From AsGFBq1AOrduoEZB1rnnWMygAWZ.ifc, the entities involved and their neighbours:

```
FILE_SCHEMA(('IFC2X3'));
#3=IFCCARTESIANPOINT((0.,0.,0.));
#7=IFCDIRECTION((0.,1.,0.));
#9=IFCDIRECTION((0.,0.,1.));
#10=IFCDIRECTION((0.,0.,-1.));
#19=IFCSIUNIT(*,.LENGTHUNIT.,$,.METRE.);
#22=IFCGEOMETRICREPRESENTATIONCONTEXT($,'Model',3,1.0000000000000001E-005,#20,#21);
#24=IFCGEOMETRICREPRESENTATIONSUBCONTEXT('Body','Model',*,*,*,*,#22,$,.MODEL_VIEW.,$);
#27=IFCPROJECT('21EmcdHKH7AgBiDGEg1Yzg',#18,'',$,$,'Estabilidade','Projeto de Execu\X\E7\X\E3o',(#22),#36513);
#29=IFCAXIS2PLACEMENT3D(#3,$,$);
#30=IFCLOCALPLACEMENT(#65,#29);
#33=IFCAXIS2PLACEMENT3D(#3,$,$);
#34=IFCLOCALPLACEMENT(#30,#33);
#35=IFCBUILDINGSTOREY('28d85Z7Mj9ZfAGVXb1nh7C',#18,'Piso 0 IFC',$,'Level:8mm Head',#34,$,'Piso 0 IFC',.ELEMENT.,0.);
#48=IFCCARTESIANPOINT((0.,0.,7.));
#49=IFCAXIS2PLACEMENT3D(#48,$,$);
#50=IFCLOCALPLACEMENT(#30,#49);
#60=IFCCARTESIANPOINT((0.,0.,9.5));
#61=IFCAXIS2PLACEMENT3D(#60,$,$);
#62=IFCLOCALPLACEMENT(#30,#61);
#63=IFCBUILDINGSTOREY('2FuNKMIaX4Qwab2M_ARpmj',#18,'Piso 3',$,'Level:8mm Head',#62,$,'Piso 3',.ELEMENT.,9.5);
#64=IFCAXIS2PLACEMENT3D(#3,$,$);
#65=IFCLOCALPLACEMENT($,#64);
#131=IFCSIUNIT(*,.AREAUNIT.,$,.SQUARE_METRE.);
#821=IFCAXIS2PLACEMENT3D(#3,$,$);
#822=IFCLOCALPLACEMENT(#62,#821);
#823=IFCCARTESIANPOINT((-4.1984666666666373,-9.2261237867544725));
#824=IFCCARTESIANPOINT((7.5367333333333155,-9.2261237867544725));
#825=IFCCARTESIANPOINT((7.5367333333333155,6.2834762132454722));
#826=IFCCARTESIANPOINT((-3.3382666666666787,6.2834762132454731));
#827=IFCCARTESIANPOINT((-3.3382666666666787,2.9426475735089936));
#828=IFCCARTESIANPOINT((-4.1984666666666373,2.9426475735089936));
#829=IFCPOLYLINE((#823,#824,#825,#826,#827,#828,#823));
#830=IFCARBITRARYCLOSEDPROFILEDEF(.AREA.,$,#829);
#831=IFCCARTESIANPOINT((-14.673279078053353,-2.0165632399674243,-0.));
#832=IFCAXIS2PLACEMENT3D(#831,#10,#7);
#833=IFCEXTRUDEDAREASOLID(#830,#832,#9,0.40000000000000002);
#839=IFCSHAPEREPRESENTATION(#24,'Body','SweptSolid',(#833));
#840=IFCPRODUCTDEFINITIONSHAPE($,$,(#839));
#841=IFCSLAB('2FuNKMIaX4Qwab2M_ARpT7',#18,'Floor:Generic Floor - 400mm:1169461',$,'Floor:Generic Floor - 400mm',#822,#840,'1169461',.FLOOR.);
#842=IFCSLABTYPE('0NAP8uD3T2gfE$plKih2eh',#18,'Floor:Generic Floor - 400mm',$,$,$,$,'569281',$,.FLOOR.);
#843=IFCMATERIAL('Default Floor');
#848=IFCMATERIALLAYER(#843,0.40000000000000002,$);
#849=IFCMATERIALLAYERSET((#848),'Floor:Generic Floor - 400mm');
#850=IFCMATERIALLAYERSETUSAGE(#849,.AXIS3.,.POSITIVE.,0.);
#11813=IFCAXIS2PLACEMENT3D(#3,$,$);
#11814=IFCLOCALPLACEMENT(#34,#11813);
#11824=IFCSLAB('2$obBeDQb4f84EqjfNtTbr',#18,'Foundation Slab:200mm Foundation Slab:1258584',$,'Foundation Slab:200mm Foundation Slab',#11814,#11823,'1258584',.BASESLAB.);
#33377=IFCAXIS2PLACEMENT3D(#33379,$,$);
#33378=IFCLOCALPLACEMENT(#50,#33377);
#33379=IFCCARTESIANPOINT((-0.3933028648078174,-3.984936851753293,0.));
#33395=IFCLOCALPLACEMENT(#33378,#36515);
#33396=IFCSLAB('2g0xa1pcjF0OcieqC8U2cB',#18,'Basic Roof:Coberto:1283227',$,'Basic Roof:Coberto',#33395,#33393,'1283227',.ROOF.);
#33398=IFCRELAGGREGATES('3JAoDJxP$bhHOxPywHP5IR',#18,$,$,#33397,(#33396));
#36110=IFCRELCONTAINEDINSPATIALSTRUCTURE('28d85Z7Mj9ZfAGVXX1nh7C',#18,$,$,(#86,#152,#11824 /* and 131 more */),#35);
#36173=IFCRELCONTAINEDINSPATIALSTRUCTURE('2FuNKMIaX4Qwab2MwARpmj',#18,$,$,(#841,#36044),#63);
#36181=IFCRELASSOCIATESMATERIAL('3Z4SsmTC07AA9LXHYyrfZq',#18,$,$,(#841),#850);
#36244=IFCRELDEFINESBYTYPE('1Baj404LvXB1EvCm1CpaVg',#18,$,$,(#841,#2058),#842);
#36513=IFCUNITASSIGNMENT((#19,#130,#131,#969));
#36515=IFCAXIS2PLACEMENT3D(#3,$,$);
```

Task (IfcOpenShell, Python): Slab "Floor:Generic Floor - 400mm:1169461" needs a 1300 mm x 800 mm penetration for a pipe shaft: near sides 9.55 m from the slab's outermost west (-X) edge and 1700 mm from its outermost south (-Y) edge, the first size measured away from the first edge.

```python
import numpy as np
import ifcopenshell
import ifcopenshell.api.feature
import ifcopenshell.api.geometry
import ifcopenshell.api.root
import ifcopenshell.geom
import ifcopenshell.util.placement
import ifcopenshell.util.representation
import ifcopenshell.util.shape
import ifcopenshell.util.unit

model = ifcopenshell.open("AsGFBq1AOrduoEZB1rnnWMygAWZ.ifc")
unit_scale = ifcopenshell.util.unit.calculate_unit_scale(model)
settings = ifcopenshell.geom.settings()


def volume(element):
    """Net volume in cubic metres, openings subtracted."""
    shape = ifcopenshell.geom.create_shape(settings, element)
    return ifcopenshell.util.shape.get_volume(shape.geometry)


slab = model.by_id(841)
before = volume(slab)

# Extent in the slab's own axes, in metres. The edges named are its -X and -Y sides.
slab_shape = ifcopenshell.geom.create_shape(settings, slab)
vertices = ifcopenshell.util.shape.get_vertices(slab_shape.geometry)
x_min, y_min, bottom = vertices.min(axis=0)
top = vertices[:, 2].max()

opening = ifcopenshell.api.root.create_entity(model, ifc_class="IfcOpeningElement", name="Pipe shaft opening")
context = ifcopenshell.util.representation.get_context(model, "Model", "Body", "MODEL_VIEW")
width, depth = 1.3, 0.8
outline = [(0.0, 0.0), (width, 0.0), (width, depth), (0.0, depth), (0.0, 0.0)]
# Overshoot both faces by 50 mm so the cut is clean.
shape = ifcopenshell.api.geometry.add_slab_representation(
    model, context=context, depth=top - bottom + 0.1, polyline=outline
)
ifcopenshell.api.geometry.assign_representation(model, product=opening, representation=shape)

matrix = ifcopenshell.util.placement.get_local_placement(slab.ObjectPlacement)
matrix[:, 3] = matrix @ np.append(np.array([x_min + 9.55, y_min + 1.7, bottom - 0.05]) / unit_scale, 1.0)
ifcopenshell.api.geometry.edit_object_placement(model, product=opening, matrix=matrix, is_si=False)
ifcopenshell.api.feature.add_feature(model, feature=opening, element=slab)

after = volume(slab)

print(f"slab volume {before:.3f} -> {after:.3f} m3")

model.write("AsGFBq1AOrduoEZB1rnnWMygAWZ_rev.ifc")
```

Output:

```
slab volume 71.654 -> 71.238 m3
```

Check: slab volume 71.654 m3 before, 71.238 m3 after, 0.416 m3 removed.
